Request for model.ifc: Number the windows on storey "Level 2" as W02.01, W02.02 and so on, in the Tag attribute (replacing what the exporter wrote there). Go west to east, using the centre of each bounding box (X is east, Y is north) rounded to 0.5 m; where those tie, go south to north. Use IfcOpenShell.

First a look at what the model holds.

```python
import ifcopenshell
import ifcopenshell.util.element
import ifcopenshell.util.placement

model = ifcopenshell.open("model.ifc")
print(model.schema)
storey = next(s for s in model.by_type("IfcBuildingStorey") if s.Name == "Level 2")
windows = [e for e in ifcopenshell.util.element.get_decomposition(storey) if e.is_a("IfcWindow")]
for e in sorted(windows, key=lambda e: e.id()):
    origin = ifcopenshell.util.placement.get_local_placement(e.ObjectPlacement)[:3, 3]
    print(e.id(), e.Tag, e.Name, origin.round(2) + 0.0, sep=" | ")
```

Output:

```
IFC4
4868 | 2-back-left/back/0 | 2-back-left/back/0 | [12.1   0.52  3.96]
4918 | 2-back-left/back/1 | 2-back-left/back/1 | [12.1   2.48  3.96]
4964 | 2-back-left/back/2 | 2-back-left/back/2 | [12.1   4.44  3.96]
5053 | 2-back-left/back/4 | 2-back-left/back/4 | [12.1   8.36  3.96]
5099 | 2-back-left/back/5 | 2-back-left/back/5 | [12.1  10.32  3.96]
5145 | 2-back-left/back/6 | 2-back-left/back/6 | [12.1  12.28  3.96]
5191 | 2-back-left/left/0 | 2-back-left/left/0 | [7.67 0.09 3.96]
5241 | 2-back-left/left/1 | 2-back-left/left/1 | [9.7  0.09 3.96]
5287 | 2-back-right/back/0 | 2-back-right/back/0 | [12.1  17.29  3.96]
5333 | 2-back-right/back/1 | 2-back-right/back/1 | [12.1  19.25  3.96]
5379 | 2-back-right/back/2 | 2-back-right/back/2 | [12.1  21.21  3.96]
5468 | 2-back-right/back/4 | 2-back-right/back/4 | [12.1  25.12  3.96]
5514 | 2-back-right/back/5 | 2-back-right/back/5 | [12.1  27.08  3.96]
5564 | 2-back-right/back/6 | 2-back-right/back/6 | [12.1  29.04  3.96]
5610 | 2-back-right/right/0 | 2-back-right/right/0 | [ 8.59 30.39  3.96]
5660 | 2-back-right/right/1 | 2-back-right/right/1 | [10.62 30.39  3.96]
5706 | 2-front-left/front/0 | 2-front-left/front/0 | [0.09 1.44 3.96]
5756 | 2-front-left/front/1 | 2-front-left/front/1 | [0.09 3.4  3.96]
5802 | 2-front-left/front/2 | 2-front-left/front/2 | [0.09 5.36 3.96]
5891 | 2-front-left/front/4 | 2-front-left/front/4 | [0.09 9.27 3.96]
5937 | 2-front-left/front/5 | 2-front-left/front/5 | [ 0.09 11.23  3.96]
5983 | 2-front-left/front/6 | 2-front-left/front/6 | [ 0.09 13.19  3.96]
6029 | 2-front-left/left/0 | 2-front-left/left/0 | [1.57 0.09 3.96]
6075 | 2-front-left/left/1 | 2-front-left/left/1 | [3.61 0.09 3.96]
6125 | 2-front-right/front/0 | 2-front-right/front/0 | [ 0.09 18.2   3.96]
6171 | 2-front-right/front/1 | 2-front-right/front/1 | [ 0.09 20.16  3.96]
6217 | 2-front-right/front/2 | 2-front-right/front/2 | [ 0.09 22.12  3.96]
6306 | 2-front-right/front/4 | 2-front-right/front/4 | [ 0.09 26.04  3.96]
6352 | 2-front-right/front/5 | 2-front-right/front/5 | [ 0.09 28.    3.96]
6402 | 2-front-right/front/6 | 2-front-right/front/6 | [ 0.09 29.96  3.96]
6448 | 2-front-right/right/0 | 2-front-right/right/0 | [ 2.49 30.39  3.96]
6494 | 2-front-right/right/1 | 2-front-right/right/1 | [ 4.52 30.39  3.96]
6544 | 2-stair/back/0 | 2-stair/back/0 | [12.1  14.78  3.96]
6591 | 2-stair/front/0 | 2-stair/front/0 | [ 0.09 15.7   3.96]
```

```python
import ifcopenshell
import ifcopenshell.geom
import ifcopenshell.util.element
import ifcopenshell.util.shape

model = ifcopenshell.open("model.ifc")
settings = ifcopenshell.geom.settings()
settings.set("use-world-coords", True)


def centre(element):
    shape = ifcopenshell.geom.create_shape(settings, element)
    return ifcopenshell.util.shape.get_bbox_centroid(shape.geometry)


storey = next(s for s in model.by_type("IfcBuildingStorey") if s.Name == "Level 2")
windows = [e for e in ifcopenshell.util.element.get_decomposition(storey) if e.is_a("IfcWindow")]

# Insertion points can sit at a corner or the storey origin, so sort by the geometry (in metres).
centres = {e: centre(e) for e in windows}
windows.sort(key=lambda e: (round(centres[e][0] / 0.5), centres[e][1]))

for i, e in enumerate(windows, start=1):
    number = f"W02.{i:02d}"
    e.Tag = number
    print(e.id(), number)

model.write("model-out.ifc")
```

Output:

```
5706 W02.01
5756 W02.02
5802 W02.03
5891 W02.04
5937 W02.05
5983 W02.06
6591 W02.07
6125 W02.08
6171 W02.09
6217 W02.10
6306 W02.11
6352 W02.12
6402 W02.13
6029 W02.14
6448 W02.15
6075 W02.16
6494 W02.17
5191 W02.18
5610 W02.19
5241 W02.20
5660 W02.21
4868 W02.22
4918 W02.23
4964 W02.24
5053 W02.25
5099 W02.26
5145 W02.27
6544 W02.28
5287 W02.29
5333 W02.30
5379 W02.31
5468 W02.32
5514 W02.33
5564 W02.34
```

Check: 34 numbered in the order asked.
